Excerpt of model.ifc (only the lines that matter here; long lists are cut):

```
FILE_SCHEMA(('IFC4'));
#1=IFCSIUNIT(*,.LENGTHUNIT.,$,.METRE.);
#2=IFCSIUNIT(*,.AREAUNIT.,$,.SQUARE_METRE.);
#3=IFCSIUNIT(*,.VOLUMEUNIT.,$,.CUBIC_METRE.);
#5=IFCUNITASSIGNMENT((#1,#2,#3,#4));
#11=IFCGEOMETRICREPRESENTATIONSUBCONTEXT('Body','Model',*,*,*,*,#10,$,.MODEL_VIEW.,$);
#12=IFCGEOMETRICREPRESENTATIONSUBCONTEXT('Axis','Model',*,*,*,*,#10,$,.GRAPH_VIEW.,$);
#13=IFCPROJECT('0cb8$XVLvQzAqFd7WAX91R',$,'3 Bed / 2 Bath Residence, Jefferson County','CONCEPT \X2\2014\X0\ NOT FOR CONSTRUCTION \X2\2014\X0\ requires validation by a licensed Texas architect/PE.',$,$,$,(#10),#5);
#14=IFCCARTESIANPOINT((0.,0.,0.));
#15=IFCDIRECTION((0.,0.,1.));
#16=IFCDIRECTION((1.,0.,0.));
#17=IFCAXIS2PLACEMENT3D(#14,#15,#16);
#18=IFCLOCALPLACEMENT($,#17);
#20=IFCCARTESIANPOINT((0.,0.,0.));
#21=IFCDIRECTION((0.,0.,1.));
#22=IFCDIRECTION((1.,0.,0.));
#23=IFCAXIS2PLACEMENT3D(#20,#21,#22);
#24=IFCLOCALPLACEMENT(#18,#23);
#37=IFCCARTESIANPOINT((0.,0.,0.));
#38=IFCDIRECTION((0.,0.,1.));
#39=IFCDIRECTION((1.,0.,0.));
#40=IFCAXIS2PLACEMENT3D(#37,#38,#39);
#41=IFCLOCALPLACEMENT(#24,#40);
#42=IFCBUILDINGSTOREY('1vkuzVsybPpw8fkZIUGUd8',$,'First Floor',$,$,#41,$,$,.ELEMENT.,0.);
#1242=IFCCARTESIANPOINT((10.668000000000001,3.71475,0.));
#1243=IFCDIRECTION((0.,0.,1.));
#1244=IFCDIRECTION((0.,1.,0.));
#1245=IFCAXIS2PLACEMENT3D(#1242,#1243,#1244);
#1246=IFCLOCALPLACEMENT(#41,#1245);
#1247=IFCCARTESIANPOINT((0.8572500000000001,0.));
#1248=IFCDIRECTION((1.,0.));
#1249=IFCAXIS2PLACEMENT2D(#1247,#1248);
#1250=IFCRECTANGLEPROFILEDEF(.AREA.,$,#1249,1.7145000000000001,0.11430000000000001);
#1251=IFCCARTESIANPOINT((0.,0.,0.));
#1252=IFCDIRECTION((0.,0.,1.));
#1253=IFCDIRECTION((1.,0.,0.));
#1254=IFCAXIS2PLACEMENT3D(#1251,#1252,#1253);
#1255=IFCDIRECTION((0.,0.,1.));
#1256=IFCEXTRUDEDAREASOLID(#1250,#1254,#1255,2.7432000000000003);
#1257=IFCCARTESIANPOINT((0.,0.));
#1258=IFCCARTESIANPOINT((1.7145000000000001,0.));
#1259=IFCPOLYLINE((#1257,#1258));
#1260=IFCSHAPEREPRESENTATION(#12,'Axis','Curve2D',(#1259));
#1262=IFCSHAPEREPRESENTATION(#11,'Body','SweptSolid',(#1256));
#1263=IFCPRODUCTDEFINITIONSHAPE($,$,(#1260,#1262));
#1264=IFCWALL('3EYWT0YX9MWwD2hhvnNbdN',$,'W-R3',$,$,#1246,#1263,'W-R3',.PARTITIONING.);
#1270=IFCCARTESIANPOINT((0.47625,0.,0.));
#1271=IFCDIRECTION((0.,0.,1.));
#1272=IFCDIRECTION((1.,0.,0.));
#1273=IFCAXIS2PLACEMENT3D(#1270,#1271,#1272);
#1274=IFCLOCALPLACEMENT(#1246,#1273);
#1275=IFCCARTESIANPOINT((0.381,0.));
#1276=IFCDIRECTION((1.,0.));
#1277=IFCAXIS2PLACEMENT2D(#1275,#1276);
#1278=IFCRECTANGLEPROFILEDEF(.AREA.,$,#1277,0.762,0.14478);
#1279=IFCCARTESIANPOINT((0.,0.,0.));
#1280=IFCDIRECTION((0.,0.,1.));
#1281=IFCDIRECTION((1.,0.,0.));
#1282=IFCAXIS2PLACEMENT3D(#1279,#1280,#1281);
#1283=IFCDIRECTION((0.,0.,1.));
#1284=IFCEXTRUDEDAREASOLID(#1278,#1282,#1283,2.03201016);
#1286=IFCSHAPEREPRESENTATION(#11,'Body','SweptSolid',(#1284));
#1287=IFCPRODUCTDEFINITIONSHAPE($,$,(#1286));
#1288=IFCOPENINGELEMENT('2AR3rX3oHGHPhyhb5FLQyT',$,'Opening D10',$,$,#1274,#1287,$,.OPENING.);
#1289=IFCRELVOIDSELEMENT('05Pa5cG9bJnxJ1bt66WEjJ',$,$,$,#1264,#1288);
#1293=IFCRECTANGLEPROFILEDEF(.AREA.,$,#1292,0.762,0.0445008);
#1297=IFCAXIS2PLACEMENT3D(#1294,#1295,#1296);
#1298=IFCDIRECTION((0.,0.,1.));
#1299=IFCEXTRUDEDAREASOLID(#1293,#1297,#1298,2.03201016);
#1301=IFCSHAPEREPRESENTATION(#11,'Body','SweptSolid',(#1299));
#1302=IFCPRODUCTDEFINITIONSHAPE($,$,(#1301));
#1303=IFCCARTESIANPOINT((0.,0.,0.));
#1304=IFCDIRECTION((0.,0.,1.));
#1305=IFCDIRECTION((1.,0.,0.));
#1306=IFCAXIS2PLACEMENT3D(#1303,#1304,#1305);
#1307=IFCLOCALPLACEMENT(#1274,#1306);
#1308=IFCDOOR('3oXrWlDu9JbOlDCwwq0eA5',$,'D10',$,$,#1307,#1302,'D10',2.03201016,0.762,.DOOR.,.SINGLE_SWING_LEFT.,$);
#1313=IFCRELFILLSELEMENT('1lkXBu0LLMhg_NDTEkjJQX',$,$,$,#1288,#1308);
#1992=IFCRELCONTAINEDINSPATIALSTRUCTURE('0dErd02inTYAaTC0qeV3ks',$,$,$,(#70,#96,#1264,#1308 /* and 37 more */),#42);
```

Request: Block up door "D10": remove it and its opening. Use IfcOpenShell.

```python
import ifcopenshell
import ifcopenshell.api.feature
import ifcopenshell.api.root
import ifcopenshell.geom
import ifcopenshell.util.shape

model = ifcopenshell.open("model.ifc")
settings = ifcopenshell.geom.settings()


def volume(element):
    """Net volume in cubic metres, openings subtracted."""
    shape = ifcopenshell.geom.create_shape(settings, element)
    return ifcopenshell.util.shape.get_volume(shape.geometry)


door = model.by_id(1308)
opening = door.FillsVoids[0].RelatingOpeningElement
wall = opening.VoidsElements[0].RelatingBuildingElement
before = volume(wall)

ifcopenshell.api.root.remove_product(model, product=door)
ifcopenshell.api.feature.remove_feature(model, feature=opening)

after = volume(wall)

print(f"wall volume {before:.3f} -> {after:.3f} m3")

model.write("model_v2.ifc")
```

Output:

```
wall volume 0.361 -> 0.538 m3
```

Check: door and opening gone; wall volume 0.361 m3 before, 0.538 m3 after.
